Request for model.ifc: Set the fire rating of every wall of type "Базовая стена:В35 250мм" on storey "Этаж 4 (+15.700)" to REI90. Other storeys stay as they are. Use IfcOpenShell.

First a look at what the model holds.

```python
import ifcopenshell
import ifcopenshell.util.element

model = ifcopenshell.open("model.ifc")
print(model.schema)
storey = next(s for s in model.by_type("IfcBuildingStorey") if s.Name == "Этаж 4 (+15.700)")
walls = [e for e in ifcopenshell.util.element.get_decomposition(storey) if e.is_a("IfcWall")]
seen = {}
for e in walls:
    element_type = ifcopenshell.util.element.get_type(e)
    key = (element_type.Name if element_type != e and element_type else None, ifcopenshell.util.element.get_pset(e, "Pset_WallCommon", "FireRating"))
    seen[key] = seen.get(key, 0) + 1
for (name, value), count in sorted(seen.items(), key=str):
    print(count, "x", name, "|", value)
```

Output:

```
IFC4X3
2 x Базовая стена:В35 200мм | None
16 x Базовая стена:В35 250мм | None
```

```python
import ifcopenshell
import ifcopenshell.api.pset
import ifcopenshell.util.element

model = ifcopenshell.open("model.ifc")

storey = next(s for s in model.by_type("IfcBuildingStorey") if s.Name == "Этаж 4 (+15.700)")
walls = [e for e in ifcopenshell.util.element.get_decomposition(storey) if e.is_a("IfcWall")]

count = 0
for e in walls:
    element_type = ifcopenshell.util.element.get_type(e)
    if element_type in (None, e) or element_type.Name != "Базовая стена:В35 250мм":
        continue
    # add_pset returns the element's existing set when there is one.
    pset = ifcopenshell.api.pset.add_pset(model, product=e, name="Pset_WallCommon")
    ifcopenshell.api.pset.edit_pset(model, pset=pset, properties={"FireRating": "REI90"})
    count += 1

print(count, "walls updated")

model.write("model_edited.ifc")
```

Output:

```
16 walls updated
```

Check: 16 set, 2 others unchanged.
